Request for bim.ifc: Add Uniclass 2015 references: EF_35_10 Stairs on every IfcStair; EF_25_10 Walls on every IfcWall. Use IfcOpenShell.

First a look at what the model holds.

```python
import ifcopenshell

model = ifcopenshell.open("bim.ifc")
print(model.schema)
print("classifications:", [c.Name for c in model.by_type("IfcClassification")])
for ifc_class in ("IfcDoor", "IfcRoof", "IfcStair", "IfcWall", "IfcWindow"):
    print(ifc_class, len(model.by_type(ifc_class)))
```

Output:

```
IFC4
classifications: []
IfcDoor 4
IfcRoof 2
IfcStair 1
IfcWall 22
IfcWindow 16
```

```python
import ifcopenshell
import ifcopenshell.api.classification

model = ifcopenshell.open("bim.ifc")

system = ifcopenshell.api.classification.add_classification(model, classification="Uniclass 2015")

codes = {
    "IfcStair": ("EF_35_10", "Stairs"),
    "IfcWall": ("EF_25_10", "Walls"),
}
for ifc_class, (code, name) in codes.items():
    products = model.by_type(ifc_class)
    ifcopenshell.api.classification.add_reference(
        model, products=products, classification=system, identification=code, name=name
    )
    print(code, len(products))

model.write("bim_updated.ifc")
```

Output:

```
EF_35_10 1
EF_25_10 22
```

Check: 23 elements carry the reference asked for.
